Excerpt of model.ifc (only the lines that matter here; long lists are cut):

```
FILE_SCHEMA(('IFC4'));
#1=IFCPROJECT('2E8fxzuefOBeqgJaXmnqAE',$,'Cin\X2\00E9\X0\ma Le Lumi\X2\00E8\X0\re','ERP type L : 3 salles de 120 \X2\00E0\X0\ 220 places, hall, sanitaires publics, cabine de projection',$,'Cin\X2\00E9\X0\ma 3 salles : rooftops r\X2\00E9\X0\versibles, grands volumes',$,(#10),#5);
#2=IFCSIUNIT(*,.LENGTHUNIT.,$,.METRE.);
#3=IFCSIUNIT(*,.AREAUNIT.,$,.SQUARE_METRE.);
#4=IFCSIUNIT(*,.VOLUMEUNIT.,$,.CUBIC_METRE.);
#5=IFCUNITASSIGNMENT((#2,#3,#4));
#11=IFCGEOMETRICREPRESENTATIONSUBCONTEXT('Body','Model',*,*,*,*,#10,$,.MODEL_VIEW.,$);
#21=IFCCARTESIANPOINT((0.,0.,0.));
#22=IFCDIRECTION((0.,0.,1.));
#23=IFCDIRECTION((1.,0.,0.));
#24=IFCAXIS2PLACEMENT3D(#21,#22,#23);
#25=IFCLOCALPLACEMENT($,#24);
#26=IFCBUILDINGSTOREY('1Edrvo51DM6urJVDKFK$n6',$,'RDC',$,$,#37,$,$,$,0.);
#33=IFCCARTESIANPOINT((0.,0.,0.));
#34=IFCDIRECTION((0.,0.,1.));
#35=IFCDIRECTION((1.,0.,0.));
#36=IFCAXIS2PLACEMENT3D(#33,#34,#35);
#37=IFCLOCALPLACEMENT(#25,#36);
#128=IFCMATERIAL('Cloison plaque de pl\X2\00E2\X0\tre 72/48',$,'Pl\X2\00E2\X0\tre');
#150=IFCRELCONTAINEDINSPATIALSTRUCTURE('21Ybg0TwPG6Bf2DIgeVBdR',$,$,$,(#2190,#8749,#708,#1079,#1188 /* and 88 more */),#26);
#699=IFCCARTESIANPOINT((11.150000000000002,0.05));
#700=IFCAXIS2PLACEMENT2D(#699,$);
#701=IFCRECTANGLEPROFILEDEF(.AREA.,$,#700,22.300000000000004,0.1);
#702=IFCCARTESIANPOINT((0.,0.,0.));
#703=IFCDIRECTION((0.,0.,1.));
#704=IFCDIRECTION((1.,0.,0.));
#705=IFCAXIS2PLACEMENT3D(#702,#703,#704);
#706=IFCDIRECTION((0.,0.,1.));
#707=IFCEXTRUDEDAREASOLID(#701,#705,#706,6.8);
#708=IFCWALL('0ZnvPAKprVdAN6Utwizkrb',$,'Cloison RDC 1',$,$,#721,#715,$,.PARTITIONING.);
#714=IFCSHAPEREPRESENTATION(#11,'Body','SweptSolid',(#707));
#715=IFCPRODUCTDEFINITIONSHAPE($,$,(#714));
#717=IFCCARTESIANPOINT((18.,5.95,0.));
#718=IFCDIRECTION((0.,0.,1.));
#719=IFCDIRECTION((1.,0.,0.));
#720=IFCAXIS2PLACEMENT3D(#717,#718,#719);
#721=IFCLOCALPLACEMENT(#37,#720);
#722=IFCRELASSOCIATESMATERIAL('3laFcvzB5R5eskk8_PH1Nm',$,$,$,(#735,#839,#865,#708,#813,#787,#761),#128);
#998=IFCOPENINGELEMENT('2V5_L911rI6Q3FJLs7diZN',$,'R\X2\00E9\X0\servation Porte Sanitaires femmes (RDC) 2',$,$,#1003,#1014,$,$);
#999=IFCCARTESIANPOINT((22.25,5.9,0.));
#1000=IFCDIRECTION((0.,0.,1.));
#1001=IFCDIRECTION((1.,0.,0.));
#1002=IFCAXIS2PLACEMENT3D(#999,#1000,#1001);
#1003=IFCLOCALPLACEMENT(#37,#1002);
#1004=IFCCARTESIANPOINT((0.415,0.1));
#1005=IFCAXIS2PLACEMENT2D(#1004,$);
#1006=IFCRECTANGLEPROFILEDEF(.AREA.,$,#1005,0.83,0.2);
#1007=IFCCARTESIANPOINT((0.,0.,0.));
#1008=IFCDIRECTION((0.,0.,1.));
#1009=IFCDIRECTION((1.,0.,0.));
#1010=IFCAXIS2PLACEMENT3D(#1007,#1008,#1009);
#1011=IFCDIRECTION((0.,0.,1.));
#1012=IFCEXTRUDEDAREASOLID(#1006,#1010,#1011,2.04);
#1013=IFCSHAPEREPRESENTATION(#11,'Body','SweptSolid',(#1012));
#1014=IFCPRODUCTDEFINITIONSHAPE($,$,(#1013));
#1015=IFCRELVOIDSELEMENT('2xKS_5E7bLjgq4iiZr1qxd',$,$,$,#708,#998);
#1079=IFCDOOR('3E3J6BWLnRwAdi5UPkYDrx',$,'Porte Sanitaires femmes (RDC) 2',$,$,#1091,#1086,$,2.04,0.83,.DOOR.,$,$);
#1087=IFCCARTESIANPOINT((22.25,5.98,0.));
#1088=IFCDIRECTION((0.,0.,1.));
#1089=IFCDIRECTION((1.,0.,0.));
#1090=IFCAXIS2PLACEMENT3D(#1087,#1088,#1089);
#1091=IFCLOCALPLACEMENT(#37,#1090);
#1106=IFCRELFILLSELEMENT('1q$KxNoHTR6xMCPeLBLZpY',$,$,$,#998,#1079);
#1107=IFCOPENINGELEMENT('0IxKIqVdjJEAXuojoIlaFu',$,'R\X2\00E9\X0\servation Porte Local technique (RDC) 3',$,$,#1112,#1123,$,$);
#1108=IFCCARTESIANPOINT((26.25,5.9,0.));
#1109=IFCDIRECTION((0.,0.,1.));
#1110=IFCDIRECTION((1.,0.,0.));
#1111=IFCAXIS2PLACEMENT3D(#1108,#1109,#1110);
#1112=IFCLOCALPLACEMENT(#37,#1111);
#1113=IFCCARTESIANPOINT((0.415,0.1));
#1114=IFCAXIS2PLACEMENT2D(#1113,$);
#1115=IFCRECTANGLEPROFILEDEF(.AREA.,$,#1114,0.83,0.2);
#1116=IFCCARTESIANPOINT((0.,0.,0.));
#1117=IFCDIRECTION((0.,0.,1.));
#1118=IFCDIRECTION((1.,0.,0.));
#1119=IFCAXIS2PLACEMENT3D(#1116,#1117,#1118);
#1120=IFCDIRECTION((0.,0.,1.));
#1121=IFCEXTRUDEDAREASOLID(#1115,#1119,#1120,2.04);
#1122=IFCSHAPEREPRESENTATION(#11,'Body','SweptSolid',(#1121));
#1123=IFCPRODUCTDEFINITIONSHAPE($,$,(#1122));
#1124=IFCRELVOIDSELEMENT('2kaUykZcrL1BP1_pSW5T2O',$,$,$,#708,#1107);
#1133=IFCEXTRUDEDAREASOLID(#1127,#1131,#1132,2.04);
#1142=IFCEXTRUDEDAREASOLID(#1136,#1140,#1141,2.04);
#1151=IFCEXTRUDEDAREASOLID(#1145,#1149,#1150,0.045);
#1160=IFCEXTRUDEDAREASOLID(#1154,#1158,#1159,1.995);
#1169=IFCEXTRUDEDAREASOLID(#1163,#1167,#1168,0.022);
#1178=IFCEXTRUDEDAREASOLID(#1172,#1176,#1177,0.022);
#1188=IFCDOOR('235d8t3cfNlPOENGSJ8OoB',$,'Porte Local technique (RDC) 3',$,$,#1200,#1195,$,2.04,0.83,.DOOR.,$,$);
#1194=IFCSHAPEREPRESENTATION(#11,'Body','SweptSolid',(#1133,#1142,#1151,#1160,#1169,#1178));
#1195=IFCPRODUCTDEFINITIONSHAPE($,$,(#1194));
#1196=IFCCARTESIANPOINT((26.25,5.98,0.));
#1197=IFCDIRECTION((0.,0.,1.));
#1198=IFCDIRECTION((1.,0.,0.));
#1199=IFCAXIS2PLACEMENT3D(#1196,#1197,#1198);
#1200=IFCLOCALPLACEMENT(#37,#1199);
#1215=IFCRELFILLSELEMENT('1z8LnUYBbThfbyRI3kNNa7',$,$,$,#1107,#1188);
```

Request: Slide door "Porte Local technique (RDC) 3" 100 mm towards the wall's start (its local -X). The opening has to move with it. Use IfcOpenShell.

```python
import ifcopenshell
import ifcopenshell.api.geometry
import ifcopenshell.util.placement

model = ifcopenshell.open("model.ifc")

door = model.by_id(1188)
opening = door.FillsVoids[0].RelatingOpeningElement
wall = opening.VoidsElements[0].RelatingBuildingElement

wall_matrix = ifcopenshell.util.placement.get_local_placement(wall.ObjectPlacement)
shift = wall_matrix[:3, 0] * -0.1
before = ifcopenshell.util.placement.get_local_placement(door.ObjectPlacement)[:3, 3].copy()

# The door is not placed relative to its opening, so move both.
for product in (opening, door):
    matrix = ifcopenshell.util.placement.get_local_placement(product.ObjectPlacement)
    matrix[:3, 3] += shift
    ifcopenshell.api.geometry.edit_object_placement(model, product=product, matrix=matrix, is_si=False)

after = ifcopenshell.util.placement.get_local_placement(door.ObjectPlacement)[:3, 3]
print("door moved by", (after - before).round(3) + 0.0)

model.write("model_updated.ifc")
```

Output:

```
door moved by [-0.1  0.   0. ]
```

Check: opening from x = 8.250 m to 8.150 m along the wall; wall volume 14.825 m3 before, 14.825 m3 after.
